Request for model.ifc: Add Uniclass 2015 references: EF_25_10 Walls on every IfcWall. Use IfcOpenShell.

First a look at what the model holds.

```python
import ifcopenshell

model = ifcopenshell.open("model.ifc")
print(model.schema)
print("classifications:", [c.Name for c in model.by_type("IfcClassification")])
for ifc_class in ("IfcDoor", "IfcRoof", "IfcStair", "IfcWall", "IfcWindow"):
    print(ifc_class, len(model.by_type(ifc_class)))
```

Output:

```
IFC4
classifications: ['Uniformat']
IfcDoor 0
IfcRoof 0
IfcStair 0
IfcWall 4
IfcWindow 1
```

```python
import ifcopenshell
import ifcopenshell.api.classification

model = ifcopenshell.open("model.ifc")

system = ifcopenshell.api.classification.add_classification(model, classification="Uniclass 2015")

codes = {
    "IfcWall": ("EF_25_10", "Walls"),
}
for ifc_class, (code, name) in codes.items():
    products = model.by_type(ifc_class)
    ifcopenshell.api.classification.add_reference(
        model, products=products, classification=system, identification=code, name=name
    )
    print(code, len(products))

model.write("model_v2.ifc")
```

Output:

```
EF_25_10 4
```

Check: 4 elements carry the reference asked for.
